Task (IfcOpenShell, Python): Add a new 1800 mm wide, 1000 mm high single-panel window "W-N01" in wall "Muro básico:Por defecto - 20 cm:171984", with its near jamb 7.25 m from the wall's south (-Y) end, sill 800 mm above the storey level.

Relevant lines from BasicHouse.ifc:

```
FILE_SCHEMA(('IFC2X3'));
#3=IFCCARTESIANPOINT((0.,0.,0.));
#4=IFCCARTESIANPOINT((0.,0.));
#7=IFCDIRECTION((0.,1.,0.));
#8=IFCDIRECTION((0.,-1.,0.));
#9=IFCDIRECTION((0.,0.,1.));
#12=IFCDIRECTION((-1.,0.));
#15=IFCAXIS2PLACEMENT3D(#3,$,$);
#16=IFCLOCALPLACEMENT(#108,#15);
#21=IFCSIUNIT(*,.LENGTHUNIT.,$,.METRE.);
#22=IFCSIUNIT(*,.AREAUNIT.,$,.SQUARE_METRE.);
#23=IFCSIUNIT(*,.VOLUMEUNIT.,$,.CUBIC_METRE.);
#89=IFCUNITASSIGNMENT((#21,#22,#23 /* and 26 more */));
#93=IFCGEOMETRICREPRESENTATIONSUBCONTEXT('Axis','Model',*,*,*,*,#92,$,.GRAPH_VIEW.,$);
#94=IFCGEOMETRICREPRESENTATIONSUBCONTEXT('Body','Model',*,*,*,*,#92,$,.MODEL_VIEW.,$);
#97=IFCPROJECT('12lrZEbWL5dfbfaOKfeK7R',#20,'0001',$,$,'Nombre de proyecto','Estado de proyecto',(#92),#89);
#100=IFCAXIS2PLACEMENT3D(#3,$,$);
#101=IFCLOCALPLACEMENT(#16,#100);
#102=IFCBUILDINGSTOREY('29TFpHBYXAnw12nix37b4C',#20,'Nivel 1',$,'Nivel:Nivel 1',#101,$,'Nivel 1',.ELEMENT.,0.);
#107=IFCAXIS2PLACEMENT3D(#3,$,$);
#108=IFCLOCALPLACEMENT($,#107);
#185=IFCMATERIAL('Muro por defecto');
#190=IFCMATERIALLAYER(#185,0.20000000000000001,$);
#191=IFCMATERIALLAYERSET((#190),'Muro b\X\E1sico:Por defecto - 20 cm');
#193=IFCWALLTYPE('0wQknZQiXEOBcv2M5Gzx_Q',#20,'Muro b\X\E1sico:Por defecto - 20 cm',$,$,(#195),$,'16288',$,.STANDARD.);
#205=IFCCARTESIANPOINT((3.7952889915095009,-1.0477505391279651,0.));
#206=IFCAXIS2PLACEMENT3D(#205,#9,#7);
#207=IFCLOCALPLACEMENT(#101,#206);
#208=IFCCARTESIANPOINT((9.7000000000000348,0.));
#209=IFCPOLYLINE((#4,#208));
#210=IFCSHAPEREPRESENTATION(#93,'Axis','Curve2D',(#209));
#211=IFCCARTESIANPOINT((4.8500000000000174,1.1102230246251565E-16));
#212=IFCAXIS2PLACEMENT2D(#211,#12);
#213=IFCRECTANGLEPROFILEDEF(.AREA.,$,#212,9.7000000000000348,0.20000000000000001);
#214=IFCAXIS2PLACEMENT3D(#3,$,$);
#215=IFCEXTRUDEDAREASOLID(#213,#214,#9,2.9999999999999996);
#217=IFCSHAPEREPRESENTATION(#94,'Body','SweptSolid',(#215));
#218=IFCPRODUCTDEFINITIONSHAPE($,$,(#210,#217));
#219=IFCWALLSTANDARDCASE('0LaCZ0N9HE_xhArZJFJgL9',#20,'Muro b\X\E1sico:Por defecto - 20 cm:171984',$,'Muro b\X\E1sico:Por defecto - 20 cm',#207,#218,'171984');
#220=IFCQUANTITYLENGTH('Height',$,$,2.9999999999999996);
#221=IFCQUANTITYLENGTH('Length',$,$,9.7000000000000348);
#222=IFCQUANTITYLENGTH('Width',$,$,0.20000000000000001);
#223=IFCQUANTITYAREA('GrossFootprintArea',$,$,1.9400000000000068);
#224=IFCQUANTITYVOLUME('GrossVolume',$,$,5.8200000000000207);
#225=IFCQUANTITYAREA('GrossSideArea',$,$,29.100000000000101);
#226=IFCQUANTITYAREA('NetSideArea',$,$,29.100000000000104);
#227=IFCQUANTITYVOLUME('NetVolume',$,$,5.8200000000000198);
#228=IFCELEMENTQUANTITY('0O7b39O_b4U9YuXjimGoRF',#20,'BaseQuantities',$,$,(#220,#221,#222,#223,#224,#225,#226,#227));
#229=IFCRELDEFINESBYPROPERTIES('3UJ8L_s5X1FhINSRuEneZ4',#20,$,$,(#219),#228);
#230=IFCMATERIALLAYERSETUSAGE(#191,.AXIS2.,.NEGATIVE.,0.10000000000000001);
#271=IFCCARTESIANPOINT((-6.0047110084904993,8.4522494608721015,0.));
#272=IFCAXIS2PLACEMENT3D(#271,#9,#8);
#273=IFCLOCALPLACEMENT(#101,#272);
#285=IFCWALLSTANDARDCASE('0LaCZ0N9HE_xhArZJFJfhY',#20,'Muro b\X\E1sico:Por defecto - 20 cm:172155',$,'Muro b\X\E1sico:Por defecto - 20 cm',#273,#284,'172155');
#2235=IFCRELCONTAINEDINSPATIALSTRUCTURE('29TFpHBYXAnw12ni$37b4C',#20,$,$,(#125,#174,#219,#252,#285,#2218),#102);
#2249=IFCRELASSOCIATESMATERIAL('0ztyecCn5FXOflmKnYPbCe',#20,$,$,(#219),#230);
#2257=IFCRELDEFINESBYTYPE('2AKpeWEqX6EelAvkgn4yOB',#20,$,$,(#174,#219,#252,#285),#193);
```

```python
import numpy as np
import ifcopenshell
import ifcopenshell.api.feature
import ifcopenshell.api.geometry
import ifcopenshell.api.pset
import ifcopenshell.api.root
import ifcopenshell.api.spatial
import ifcopenshell.api.type
import ifcopenshell.geom
import ifcopenshell.util.element
import ifcopenshell.util.placement
import ifcopenshell.util.representation
import ifcopenshell.util.shape
import ifcopenshell.util.unit

model = ifcopenshell.open("BasicHouse.ifc")
unit_scale = ifcopenshell.util.unit.calculate_unit_scale(model)
area_scale = ifcopenshell.util.unit.calculate_unit_scale(model, "AREAUNIT")
volume_scale = ifcopenshell.util.unit.calculate_unit_scale(model, "VOLUMEUNIT")
settings = ifcopenshell.geom.settings()


def volume(element):
    """Net volume in cubic metres, openings subtracted."""
    shape = ifcopenshell.geom.create_shape(settings, element)
    return ifcopenshell.util.shape.get_volume(shape.geometry)


wall = model.by_id(219)
storey = ifcopenshell.util.element.get_container(wall, ifc_class="IfcBuildingStorey")
context = ifcopenshell.util.representation.get_context(model, "Model", "Body", "MODEL_VIEW")
before = volume(wall)

width, height, from_end, sill = 1.8, 1, 7.25, 0.8  # metres

# The wall runs along its own X axis, and the end named is its -X end.
wall_shape = ifcopenshell.geom.create_shape(settings, wall)
x, y, z = ifcopenshell.util.shape.get_vertices(wall_shape.geometry).T
start = x.min() + from_end
face, thickness = float(y.min()), float(y.max() - y.min())
wall_matrix = ifcopenshell.util.placement.get_local_placement(wall.ObjectPlacement)
level = ifcopenshell.util.placement.get_local_placement(storey.ObjectPlacement)[2, 3]


def in_wall(x, y):
    """Placement at x, y metres in the wall's axes, at sill height."""
    matrix = wall_matrix.copy()
    matrix[:, 3] = wall_matrix @ np.array([x / unit_scale, y / unit_scale, 0.0, 1.0])
    matrix[2, 3] = level + sill / unit_scale
    return matrix


# Opening: a box that overshoots both wall faces by 50 mm.
opening = ifcopenshell.api.root.create_entity(model, ifc_class="IfcOpeningElement")
box = ifcopenshell.api.geometry.add_wall_representation(
    model, context=context, length=width, height=height, thickness=thickness + 0.1
)
ifcopenshell.api.geometry.assign_representation(model, product=opening, representation=box)
ifcopenshell.api.geometry.edit_object_placement(model, product=opening, matrix=in_wall(start, face - 0.05), is_si=False)
ifcopenshell.api.feature.add_feature(model, feature=opening, element=wall)

window = ifcopenshell.api.root.create_entity(model, ifc_class="IfcWindow", name="W-N01")
window.OverallWidth, window.OverallHeight = width / unit_scale, height / unit_scale
body = ifcopenshell.api.geometry.add_window_representation(
    model,
    context=context,
    overall_width=window.OverallWidth,
    overall_height=window.OverallHeight,
    partition_type="SINGLE_PANEL",
)
ifcopenshell.api.geometry.assign_representation(model, product=window, representation=body)
ifcopenshell.api.spatial.assign_container(model, products=[window], relating_structure=storey)
fills = ifcopenshell.api.feature.add_filling(model, opening=opening, element=window)
fills.OwnerHistory = window.OwnerHistory  # required in IFC2X3

# IFC2X3 keeps the operation on the window style.
style = ifcopenshell.api.root.create_entity(model, ifc_class="IfcWindowStyle", name="W-N01")
style.OperationType, style.ConstructionType = "SINGLE_PANEL", "NOTDEFINED"
style.ParameterTakesPrecedence = style.Sizeable = False
ifcopenshell.api.type.assign_type(model, related_objects=[window], relating_type=style)

# Centre the window in the wall's thickness.
ifcopenshell.api.geometry.edit_object_placement(model, product=window, matrix=in_wall(start, face), is_si=False)
window_shape = ifcopenshell.geom.create_shape(settings, window)
depth = ifcopenshell.util.shape.get_vertices(window_shape.geometry)[:, 1]
offset = face + thickness / 2 - (depth.min() + depth.max()) / 2
ifcopenshell.api.geometry.edit_object_placement(model, product=window, matrix=in_wall(start, offset), is_si=False)

after = volume(wall)

# Update the wall's stored quantities.
qto = model.by_id(ifcopenshell.util.element.get_pset(wall, "BaseQuantities", should_inherit=False)["id"])
ifcopenshell.api.pset.edit_qto(model, qto=qto, properties={
    "NetSideArea": after / thickness / area_scale,
    "NetVolume": after / volume_scale,
})

print(f"wall volume {before:.3f} -> {after:.3f} m3")

model.write("BasicHouse_rev.ifc")
```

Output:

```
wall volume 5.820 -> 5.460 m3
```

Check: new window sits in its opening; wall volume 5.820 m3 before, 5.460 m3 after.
